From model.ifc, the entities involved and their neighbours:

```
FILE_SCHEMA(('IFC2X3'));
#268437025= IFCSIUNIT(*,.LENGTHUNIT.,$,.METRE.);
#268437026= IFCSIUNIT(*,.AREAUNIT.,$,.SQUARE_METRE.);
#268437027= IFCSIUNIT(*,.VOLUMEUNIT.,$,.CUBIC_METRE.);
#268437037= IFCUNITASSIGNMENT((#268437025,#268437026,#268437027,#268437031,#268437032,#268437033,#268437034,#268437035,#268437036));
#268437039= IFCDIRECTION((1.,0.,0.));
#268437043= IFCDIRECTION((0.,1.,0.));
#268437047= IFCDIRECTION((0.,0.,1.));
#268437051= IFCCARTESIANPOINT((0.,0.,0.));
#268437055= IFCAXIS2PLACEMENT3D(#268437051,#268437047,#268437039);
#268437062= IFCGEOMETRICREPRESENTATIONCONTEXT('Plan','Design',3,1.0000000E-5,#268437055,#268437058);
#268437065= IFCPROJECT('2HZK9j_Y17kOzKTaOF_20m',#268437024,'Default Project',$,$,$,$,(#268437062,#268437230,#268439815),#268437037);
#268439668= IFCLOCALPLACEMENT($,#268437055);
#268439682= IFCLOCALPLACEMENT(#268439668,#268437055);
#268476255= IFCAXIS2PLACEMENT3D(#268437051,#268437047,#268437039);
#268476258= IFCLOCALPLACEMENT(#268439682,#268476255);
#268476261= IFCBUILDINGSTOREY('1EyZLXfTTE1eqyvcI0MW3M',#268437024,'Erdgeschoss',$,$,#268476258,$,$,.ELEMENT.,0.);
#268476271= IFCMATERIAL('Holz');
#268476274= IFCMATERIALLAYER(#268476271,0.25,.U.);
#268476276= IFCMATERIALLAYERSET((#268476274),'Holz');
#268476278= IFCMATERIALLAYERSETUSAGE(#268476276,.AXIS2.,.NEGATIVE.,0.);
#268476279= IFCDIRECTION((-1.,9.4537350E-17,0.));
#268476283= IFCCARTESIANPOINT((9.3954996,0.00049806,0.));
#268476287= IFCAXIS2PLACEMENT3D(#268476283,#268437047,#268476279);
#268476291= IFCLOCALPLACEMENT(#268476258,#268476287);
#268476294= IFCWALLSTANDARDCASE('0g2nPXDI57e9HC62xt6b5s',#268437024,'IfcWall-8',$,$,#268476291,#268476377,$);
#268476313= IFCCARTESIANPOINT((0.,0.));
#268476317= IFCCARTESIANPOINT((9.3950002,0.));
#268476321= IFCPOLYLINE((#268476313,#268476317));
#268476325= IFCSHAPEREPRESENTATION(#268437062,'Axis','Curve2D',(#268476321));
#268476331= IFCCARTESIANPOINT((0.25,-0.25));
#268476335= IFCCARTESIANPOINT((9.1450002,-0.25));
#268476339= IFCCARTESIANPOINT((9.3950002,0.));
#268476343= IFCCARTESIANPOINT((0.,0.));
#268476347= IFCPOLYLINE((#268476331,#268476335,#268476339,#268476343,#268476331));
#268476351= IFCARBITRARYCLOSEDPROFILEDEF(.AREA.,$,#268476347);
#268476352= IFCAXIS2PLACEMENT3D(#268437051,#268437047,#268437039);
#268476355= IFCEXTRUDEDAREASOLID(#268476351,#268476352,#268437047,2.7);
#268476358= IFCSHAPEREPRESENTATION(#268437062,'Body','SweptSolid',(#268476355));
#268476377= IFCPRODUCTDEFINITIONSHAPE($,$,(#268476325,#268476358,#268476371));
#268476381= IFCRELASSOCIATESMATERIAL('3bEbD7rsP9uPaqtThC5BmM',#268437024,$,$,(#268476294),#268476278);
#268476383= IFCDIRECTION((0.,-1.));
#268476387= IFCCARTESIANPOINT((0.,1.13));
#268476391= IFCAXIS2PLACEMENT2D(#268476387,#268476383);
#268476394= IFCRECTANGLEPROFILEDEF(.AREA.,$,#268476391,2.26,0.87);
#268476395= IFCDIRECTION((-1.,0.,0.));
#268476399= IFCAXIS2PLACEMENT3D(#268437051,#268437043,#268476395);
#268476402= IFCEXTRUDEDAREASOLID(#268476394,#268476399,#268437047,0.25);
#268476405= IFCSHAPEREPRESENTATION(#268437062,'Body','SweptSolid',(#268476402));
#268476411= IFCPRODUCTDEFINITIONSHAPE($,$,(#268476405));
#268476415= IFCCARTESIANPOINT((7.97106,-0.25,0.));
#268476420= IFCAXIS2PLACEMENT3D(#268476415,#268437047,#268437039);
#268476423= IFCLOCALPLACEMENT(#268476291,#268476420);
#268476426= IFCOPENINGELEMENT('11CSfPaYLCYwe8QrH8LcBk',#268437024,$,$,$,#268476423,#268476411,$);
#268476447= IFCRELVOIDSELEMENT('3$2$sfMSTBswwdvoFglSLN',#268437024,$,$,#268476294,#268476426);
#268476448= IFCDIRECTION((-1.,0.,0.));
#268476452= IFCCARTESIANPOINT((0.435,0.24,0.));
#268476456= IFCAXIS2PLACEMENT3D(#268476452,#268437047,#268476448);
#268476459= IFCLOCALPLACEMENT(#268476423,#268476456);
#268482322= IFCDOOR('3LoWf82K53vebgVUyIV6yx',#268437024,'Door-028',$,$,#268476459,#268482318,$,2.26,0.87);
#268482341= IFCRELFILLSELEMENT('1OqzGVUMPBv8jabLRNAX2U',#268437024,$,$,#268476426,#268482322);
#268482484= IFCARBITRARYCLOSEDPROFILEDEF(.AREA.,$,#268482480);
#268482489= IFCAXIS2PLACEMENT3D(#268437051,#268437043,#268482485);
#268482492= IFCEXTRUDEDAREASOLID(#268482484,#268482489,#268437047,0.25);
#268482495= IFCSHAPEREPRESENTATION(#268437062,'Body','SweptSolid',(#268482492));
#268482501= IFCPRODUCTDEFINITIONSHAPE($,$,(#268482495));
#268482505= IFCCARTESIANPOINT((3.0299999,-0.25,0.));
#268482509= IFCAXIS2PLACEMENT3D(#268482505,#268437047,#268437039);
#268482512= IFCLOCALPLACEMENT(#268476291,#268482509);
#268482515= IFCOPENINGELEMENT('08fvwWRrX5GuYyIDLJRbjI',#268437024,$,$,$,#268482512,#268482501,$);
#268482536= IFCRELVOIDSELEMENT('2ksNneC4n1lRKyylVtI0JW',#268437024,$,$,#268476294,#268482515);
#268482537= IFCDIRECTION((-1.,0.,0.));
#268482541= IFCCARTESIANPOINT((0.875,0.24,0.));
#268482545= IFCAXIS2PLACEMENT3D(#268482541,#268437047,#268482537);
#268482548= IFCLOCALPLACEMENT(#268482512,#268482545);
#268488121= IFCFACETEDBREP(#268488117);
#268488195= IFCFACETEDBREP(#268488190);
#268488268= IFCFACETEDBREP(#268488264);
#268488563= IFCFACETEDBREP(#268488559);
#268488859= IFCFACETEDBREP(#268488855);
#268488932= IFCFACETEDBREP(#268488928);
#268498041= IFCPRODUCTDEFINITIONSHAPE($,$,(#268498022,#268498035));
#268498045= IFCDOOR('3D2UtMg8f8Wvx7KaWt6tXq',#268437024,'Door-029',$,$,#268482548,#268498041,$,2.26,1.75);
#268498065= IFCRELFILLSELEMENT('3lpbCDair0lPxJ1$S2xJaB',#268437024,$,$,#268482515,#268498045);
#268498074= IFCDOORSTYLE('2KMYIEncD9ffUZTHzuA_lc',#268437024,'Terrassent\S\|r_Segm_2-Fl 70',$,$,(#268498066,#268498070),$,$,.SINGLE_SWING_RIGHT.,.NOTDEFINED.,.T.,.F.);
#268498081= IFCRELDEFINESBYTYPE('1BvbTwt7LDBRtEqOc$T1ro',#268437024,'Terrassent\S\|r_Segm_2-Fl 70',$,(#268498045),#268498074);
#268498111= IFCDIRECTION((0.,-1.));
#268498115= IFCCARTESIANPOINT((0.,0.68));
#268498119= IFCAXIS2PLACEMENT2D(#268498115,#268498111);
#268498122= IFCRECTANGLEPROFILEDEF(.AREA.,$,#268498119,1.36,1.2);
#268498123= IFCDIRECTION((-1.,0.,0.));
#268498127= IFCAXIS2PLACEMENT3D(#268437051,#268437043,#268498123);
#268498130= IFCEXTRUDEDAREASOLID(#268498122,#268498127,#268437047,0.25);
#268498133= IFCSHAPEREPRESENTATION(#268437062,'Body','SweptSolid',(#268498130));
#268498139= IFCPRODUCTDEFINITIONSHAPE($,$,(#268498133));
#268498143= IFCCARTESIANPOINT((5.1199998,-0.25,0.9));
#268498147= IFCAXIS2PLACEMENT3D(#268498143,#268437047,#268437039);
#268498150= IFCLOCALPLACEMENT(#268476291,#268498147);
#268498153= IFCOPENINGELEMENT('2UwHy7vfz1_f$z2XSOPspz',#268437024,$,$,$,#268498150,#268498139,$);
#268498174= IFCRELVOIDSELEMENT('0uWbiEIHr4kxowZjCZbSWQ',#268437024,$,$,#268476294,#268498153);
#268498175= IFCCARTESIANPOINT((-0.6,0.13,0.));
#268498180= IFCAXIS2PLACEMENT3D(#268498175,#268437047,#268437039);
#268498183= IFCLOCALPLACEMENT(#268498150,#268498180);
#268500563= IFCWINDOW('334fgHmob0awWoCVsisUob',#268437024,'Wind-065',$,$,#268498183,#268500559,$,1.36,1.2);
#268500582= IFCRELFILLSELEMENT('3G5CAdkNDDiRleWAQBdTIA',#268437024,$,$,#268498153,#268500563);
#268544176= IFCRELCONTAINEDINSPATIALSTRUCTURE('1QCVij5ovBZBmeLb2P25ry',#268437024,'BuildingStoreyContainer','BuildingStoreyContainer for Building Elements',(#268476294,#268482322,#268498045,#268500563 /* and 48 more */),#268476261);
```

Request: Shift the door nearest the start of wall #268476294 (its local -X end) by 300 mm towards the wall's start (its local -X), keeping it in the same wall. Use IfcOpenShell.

```python
import ifcopenshell
import ifcopenshell.api.geometry
import ifcopenshell.util.placement
import ifcopenshell.util.unit

model = ifcopenshell.open("model.ifc")
unit_scale = ifcopenshell.util.unit.calculate_unit_scale(model)

door = model.by_guid("3D2UtMg8f8Wvx7KaWt6tXq")
opening = door.FillsVoids[0].RelatingOpeningElement
wall = opening.VoidsElements[0].RelatingBuildingElement

wall_matrix = ifcopenshell.util.placement.get_local_placement(wall.ObjectPlacement)
shift = wall_matrix[:3, 0] * -0.3 / unit_scale
before = ifcopenshell.util.placement.get_local_placement(door.ObjectPlacement)[:3, 3].copy()

# The door is placed relative to its opening, so it follows when the opening moves.
matrix = ifcopenshell.util.placement.get_local_placement(opening.ObjectPlacement)
matrix[:3, 3] += shift
ifcopenshell.api.geometry.edit_object_placement(
    model, product=opening, matrix=matrix, is_si=False, should_transform_children=True
)

after = ifcopenshell.util.placement.get_local_placement(door.ObjectPlacement)[:3, 3]
print("door moved by", (after - before).round(3) + 0.0)

model.write("model_edited.ifc")
```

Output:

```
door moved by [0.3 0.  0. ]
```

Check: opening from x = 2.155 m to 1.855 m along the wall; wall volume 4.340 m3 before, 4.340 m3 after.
